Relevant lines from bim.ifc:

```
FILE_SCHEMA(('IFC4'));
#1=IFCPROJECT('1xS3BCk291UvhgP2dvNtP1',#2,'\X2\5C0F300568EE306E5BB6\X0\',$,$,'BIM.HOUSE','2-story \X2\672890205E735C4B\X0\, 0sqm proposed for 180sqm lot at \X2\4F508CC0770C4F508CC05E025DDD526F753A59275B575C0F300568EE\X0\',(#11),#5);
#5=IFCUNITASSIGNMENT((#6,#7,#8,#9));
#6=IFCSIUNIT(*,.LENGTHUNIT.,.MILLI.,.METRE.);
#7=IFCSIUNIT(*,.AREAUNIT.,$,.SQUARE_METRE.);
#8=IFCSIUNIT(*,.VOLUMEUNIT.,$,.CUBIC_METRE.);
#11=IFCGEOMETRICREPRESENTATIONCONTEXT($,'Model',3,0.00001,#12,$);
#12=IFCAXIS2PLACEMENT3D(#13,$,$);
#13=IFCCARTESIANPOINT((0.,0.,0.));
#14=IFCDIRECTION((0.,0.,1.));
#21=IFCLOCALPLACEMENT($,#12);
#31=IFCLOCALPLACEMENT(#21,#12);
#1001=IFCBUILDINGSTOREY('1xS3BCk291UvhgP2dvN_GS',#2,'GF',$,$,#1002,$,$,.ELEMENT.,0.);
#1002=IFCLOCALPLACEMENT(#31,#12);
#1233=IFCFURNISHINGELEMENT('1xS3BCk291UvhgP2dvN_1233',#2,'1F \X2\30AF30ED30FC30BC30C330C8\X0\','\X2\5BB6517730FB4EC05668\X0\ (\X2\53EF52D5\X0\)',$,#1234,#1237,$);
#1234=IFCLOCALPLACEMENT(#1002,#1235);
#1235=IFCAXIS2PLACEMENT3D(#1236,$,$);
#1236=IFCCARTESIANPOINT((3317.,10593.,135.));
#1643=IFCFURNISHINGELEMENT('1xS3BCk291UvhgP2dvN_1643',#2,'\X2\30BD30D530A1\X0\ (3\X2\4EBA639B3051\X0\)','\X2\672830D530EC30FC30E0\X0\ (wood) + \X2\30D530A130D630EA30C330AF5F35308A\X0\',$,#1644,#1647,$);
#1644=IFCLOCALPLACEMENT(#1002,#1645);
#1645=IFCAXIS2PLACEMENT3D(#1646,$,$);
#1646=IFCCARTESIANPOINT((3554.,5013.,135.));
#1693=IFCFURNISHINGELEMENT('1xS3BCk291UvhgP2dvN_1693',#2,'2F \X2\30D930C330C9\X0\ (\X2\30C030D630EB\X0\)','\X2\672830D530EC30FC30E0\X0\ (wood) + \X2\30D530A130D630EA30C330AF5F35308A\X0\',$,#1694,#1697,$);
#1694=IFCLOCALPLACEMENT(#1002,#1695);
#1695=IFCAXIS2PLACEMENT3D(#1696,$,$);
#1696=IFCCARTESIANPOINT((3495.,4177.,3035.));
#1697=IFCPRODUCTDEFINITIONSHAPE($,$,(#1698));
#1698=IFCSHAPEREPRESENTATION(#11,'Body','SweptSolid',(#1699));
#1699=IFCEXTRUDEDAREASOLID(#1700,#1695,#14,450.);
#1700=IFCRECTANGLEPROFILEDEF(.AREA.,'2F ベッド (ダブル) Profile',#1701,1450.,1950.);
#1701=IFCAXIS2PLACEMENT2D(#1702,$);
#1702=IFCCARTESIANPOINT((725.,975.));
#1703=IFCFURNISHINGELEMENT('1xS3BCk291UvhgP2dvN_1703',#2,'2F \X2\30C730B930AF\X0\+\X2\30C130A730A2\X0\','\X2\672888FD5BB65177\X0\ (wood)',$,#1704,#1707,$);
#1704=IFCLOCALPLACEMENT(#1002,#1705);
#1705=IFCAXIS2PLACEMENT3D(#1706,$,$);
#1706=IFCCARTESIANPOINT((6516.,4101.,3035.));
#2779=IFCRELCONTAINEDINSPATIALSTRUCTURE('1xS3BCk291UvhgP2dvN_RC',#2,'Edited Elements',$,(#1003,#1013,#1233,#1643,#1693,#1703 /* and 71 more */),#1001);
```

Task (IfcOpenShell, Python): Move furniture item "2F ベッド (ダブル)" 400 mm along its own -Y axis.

```python
import ifcopenshell
import ifcopenshell.api.geometry
import ifcopenshell.util.placement
import ifcopenshell.util.unit

model = ifcopenshell.open("bim.ifc")
unit_scale = ifcopenshell.util.unit.calculate_unit_scale(model)

item = model.by_guid("1xS3BCk291UvhgP2dvN_1693")
matrix = ifcopenshell.util.placement.get_local_placement(item.ObjectPlacement)
matrix[:3, 3] -= matrix[:3, 1] * 0.4 / unit_scale
ifcopenshell.api.geometry.edit_object_placement(model, product=item, matrix=matrix, is_si=False)

print(ifcopenshell.util.placement.get_local_placement(item.ObjectPlacement).round(3) + 0.0)

model.write("bim_rev.ifc")
```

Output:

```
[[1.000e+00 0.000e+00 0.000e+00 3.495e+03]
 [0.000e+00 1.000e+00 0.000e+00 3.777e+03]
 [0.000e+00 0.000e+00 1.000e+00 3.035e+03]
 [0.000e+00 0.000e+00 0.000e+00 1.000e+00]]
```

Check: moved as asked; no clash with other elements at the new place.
